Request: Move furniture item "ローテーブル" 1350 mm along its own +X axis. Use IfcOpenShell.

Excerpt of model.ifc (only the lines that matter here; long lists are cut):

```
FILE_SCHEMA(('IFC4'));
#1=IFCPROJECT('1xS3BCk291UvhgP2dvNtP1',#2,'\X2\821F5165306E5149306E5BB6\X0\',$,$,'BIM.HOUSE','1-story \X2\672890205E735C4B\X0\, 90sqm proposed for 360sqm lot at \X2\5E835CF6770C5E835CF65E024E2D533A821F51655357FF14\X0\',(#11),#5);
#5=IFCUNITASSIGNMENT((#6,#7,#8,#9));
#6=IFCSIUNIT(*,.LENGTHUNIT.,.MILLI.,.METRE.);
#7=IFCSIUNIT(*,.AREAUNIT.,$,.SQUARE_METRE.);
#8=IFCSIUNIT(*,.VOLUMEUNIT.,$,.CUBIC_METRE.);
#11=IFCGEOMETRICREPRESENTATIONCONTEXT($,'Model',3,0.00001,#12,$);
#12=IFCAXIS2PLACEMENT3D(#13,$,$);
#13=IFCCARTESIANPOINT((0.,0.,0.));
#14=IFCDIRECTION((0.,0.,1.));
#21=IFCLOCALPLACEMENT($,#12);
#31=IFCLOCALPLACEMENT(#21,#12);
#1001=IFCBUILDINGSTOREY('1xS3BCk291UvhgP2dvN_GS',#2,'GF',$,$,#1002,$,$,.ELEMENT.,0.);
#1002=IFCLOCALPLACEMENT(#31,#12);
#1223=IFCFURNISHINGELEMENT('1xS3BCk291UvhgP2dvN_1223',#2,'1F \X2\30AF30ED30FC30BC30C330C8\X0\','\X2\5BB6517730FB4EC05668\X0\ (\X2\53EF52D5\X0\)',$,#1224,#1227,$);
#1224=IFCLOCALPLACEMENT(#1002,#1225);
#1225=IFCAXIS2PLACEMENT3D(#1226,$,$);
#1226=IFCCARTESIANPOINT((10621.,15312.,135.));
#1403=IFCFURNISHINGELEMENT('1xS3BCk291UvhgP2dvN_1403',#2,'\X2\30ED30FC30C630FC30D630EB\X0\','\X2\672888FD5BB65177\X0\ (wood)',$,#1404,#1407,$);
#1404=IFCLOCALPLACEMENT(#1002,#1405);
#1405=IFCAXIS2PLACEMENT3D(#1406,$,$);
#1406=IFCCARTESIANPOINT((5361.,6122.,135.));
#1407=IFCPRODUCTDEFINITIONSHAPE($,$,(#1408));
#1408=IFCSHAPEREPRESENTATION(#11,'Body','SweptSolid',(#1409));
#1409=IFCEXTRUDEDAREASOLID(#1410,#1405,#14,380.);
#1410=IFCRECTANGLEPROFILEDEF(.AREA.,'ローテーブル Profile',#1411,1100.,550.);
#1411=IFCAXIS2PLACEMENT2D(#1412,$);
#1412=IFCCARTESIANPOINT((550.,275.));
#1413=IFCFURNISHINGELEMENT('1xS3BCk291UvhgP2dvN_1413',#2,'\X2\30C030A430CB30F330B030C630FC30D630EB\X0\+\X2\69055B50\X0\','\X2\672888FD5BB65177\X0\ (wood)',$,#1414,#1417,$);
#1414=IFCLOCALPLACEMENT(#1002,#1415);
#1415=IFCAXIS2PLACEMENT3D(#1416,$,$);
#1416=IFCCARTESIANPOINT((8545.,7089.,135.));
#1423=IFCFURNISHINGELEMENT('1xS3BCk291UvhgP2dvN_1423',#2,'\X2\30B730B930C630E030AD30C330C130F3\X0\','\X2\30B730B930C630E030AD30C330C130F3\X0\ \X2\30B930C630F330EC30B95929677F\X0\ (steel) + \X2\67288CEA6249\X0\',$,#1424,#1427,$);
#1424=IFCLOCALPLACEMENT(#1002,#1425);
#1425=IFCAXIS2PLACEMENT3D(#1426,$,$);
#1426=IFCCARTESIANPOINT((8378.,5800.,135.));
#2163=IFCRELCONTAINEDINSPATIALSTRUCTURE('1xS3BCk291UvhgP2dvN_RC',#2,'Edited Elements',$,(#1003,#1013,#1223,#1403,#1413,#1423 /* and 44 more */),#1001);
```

```python
import ifcopenshell
import ifcopenshell.api.geometry
import ifcopenshell.util.placement
import ifcopenshell.util.unit

model = ifcopenshell.open("model.ifc")
unit_scale = ifcopenshell.util.unit.calculate_unit_scale(model)

item = model.by_guid("1xS3BCk291UvhgP2dvN_1403")
matrix = ifcopenshell.util.placement.get_local_placement(item.ObjectPlacement)
matrix[:3, 3] += matrix[:3, 0] * 1.35 / unit_scale
ifcopenshell.api.geometry.edit_object_placement(model, product=item, matrix=matrix, is_si=False)

print(ifcopenshell.util.placement.get_local_placement(item.ObjectPlacement).round(3) + 0.0)

model.write("model-out.ifc")
```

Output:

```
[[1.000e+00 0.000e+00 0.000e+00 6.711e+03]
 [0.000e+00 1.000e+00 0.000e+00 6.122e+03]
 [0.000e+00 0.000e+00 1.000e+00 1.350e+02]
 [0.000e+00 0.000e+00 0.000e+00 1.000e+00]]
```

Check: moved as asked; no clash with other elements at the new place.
